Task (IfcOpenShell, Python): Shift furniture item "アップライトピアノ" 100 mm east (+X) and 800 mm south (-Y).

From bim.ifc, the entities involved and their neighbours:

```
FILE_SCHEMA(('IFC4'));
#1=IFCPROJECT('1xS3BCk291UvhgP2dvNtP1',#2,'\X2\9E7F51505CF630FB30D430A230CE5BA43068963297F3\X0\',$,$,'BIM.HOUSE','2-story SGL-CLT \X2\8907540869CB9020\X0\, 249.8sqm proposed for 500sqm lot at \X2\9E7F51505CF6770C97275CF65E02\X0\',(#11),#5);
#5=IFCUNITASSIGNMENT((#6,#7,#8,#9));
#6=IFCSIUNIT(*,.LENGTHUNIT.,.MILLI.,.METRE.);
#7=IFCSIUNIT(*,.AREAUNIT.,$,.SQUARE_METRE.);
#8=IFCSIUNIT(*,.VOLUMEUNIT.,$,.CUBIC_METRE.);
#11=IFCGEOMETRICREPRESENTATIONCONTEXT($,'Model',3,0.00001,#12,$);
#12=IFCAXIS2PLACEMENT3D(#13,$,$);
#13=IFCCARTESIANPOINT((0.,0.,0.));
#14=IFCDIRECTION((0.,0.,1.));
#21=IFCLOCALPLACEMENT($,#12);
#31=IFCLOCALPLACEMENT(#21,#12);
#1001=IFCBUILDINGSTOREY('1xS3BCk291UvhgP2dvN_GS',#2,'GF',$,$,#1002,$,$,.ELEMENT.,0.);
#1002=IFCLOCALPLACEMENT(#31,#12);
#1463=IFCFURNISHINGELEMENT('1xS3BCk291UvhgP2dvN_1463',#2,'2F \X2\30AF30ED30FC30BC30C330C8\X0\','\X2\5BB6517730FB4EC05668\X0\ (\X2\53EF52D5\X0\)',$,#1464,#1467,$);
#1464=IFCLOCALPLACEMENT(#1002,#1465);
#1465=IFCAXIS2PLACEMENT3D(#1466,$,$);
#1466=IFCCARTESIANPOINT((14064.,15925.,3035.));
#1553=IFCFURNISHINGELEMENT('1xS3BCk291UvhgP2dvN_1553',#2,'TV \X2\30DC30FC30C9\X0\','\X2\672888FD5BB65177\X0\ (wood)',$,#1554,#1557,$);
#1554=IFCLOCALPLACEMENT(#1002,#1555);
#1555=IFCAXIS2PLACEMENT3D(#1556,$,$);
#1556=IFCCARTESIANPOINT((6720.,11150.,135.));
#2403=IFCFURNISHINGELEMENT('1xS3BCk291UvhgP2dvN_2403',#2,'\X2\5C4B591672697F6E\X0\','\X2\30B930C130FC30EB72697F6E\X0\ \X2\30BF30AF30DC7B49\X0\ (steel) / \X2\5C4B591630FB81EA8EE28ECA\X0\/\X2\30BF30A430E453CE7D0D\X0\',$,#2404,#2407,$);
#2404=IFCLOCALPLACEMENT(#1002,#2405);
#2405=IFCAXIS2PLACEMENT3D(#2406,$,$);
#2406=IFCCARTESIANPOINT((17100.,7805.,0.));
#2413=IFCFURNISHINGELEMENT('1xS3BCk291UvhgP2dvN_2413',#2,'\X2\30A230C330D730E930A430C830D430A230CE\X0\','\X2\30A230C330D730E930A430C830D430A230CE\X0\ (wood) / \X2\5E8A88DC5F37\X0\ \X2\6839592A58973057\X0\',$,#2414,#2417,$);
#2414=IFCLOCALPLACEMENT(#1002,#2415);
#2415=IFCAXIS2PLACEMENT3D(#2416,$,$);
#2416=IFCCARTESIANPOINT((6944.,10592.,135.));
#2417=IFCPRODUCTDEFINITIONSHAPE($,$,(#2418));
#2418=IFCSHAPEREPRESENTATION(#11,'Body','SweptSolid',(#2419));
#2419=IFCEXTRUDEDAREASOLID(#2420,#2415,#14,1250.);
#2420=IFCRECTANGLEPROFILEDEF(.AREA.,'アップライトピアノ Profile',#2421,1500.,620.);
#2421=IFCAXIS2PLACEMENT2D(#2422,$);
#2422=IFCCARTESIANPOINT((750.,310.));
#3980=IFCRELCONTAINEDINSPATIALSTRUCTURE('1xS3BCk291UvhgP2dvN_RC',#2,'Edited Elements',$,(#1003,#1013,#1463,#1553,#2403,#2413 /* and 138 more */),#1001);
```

```python
import ifcopenshell
import ifcopenshell.api.geometry
import ifcopenshell.util.placement
import ifcopenshell.util.unit

model = ifcopenshell.open("bim.ifc")
unit_scale = ifcopenshell.util.unit.calculate_unit_scale(model)

item = model.by_guid("1xS3BCk291UvhgP2dvN_2413")
matrix = ifcopenshell.util.placement.get_local_placement(item.ObjectPlacement)
matrix[0, 3] += 0.1 / unit_scale
matrix[1, 3] -= 0.8 / unit_scale
ifcopenshell.api.geometry.edit_object_placement(model, product=item, matrix=matrix, is_si=False)

print(ifcopenshell.util.placement.get_local_placement(item.ObjectPlacement).round(3) + 0.0)

model.write("bim_v2.ifc")
```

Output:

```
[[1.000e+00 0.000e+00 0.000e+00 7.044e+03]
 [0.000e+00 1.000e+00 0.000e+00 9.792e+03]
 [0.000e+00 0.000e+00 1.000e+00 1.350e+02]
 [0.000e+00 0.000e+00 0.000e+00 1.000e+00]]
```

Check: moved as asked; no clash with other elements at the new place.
